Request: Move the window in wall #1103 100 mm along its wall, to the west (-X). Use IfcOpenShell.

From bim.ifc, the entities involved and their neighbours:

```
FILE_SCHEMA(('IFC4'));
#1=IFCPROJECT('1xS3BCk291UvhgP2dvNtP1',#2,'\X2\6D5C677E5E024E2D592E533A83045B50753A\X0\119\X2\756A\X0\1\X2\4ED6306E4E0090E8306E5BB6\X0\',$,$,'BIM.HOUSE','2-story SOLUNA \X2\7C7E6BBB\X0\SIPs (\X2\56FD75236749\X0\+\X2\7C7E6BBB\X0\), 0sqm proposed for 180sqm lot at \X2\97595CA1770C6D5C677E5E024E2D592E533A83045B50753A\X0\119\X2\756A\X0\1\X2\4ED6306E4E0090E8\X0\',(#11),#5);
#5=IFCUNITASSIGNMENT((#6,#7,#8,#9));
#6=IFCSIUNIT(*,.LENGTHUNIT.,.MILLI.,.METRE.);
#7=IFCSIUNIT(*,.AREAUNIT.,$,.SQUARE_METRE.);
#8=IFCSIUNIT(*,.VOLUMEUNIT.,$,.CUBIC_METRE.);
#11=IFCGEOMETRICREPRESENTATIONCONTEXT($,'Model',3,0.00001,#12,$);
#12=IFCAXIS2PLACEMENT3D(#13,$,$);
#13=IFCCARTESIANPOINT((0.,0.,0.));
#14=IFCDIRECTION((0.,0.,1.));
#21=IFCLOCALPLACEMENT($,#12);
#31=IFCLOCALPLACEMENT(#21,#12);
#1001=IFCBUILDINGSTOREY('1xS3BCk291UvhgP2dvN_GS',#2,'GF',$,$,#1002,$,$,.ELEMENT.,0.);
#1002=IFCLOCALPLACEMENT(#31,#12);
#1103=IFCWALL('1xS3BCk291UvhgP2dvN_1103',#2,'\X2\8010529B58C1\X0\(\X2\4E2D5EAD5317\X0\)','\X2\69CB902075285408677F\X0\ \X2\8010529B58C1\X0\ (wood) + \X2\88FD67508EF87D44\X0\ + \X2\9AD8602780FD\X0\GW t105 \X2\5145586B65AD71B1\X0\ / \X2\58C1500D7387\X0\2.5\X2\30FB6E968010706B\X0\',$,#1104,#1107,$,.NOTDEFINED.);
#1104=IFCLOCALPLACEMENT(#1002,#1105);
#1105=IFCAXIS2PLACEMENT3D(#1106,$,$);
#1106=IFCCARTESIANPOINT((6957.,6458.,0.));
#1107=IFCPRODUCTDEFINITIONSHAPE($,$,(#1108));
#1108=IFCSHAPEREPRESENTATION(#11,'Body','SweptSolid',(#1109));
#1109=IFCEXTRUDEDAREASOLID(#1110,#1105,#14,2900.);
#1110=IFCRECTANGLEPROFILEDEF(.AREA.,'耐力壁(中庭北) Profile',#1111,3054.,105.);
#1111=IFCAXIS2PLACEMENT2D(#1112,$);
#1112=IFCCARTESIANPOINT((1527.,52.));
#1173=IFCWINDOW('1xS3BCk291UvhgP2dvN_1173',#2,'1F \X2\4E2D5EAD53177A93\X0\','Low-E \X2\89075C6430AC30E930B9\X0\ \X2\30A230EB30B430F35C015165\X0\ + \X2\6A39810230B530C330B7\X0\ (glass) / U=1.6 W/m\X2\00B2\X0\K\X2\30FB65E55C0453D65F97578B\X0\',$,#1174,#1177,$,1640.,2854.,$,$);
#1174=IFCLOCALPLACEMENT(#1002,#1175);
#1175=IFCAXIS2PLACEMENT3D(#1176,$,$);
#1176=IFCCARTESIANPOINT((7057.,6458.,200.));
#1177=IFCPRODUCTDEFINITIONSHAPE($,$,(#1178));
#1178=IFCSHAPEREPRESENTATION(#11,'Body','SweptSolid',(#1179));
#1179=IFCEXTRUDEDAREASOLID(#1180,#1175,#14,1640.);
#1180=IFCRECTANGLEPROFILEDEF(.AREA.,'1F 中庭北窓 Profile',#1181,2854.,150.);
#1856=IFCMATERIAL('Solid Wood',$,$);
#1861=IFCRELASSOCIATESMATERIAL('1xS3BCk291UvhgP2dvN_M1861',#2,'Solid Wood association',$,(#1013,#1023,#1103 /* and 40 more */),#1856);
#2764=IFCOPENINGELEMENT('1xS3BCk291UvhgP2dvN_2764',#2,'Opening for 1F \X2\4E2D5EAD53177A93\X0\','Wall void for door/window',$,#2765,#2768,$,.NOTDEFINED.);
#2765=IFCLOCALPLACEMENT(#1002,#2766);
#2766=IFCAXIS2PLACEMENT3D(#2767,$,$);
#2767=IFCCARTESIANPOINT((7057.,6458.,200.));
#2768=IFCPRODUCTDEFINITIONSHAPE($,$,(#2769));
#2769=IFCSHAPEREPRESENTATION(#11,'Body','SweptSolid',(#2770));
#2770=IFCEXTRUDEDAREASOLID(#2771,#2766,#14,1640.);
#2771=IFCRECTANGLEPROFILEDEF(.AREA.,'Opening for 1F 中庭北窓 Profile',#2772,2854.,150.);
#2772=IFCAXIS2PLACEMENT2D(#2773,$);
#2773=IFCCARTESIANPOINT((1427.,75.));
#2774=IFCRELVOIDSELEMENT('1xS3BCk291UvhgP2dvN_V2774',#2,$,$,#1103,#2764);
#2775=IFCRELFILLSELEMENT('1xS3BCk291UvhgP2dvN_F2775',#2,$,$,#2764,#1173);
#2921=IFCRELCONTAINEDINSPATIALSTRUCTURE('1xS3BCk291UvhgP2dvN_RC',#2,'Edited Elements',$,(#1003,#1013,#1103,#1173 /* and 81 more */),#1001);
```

```python
import ifcopenshell
import ifcopenshell.api.geometry
import ifcopenshell.util.placement
import ifcopenshell.util.unit

model = ifcopenshell.open("bim.ifc")
unit_scale = ifcopenshell.util.unit.calculate_unit_scale(model)

window = model.by_id(1173)
opening = window.FillsVoids[0].RelatingOpeningElement
wall = opening.VoidsElements[0].RelatingBuildingElement

wall_matrix = ifcopenshell.util.placement.get_local_placement(wall.ObjectPlacement)
shift = wall_matrix[:3, 0] * -0.1 / unit_scale
before = ifcopenshell.util.placement.get_local_placement(window.ObjectPlacement)[:3, 3].copy()

# The window is not placed relative to its opening, so move both.
for product in (opening, window):
    matrix = ifcopenshell.util.placement.get_local_placement(product.ObjectPlacement)
    matrix[:3, 3] += shift
    ifcopenshell.api.geometry.edit_object_placement(model, product=product, matrix=matrix, is_si=False)

after = ifcopenshell.util.placement.get_local_placement(window.ObjectPlacement)[:3, 3]
print("window moved by", (after - before).round(3) + 0.0)

model.write("bim_updated.ifc")
```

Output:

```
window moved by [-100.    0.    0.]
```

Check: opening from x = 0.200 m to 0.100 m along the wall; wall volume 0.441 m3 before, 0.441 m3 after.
